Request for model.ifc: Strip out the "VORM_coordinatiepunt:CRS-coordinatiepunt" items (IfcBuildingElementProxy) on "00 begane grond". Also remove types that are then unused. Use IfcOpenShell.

First a look at what the model holds.

```python
import ifcopenshell
import ifcopenshell.util.element

model = ifcopenshell.open("model.ifc")
print(model.schema)
storey = next(s for s in model.by_type("IfcBuildingStorey") if s.Name == "00 begane grond")
proxies = [e for e in ifcopenshell.util.element.get_decomposition(storey) if e.is_a("IfcBuildingElementProxy")]
seen = {}
for e in proxies:
    element_type = ifcopenshell.util.element.get_type(e)
    name = element_type.Name if element_type not in (None, e) else None
    seen[name] = seen.get(name, 0) + 1
for name, count in sorted(seen.items(), key=str):
    print(count, "x", name)
```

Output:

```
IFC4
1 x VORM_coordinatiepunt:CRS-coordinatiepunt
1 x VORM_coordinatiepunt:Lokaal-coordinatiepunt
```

```python
import ifcopenshell
import ifcopenshell.api.root
import ifcopenshell.util.element

model = ifcopenshell.open("model.ifc")

storey = next(s for s in model.by_type("IfcBuildingStorey") if s.Name == "00 begane grond")
proxies = [e for e in ifcopenshell.util.element.get_decomposition(storey) if e.is_a("IfcBuildingElementProxy")]
targets = [e for e in proxies if (t := ifcopenshell.util.element.get_type(e)) not in (None, e) and t.Name == "VORM_coordinatiepunt:CRS-coordinatiepunt"]
types = {ifcopenshell.util.element.get_type(e) for e in targets} - {None, *targets}

for e in targets:
    ifcopenshell.api.root.remove_product(model, product=e)
print(len(targets), "removed")

unused = [t for t in types if not ifcopenshell.util.element.get_types(t)]
for t in unused:
    ifcopenshell.api.root.remove_product(model, product=t)
print(len(unused), "unused types removed")

model.write("model_updated.ifc")
```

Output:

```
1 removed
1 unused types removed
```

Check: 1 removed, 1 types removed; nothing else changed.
